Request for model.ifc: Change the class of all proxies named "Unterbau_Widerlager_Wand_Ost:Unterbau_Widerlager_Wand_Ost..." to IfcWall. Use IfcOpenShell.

First a look at what the model holds.

```python
import re

import ifcopenshell

model = ifcopenshell.open("model.ifc")
print(model.schema)
seen = {}
for e in model.by_type("IfcBuildingElementProxy"):
    name = re.sub(r":\d+(:\d+)?$", "", e.Name or "")  # drop the element id that some exporters append
    seen[name] = seen.get(name, 0) + 1
for name, count in sorted(seen.items()):
    print(count, "x", name)
```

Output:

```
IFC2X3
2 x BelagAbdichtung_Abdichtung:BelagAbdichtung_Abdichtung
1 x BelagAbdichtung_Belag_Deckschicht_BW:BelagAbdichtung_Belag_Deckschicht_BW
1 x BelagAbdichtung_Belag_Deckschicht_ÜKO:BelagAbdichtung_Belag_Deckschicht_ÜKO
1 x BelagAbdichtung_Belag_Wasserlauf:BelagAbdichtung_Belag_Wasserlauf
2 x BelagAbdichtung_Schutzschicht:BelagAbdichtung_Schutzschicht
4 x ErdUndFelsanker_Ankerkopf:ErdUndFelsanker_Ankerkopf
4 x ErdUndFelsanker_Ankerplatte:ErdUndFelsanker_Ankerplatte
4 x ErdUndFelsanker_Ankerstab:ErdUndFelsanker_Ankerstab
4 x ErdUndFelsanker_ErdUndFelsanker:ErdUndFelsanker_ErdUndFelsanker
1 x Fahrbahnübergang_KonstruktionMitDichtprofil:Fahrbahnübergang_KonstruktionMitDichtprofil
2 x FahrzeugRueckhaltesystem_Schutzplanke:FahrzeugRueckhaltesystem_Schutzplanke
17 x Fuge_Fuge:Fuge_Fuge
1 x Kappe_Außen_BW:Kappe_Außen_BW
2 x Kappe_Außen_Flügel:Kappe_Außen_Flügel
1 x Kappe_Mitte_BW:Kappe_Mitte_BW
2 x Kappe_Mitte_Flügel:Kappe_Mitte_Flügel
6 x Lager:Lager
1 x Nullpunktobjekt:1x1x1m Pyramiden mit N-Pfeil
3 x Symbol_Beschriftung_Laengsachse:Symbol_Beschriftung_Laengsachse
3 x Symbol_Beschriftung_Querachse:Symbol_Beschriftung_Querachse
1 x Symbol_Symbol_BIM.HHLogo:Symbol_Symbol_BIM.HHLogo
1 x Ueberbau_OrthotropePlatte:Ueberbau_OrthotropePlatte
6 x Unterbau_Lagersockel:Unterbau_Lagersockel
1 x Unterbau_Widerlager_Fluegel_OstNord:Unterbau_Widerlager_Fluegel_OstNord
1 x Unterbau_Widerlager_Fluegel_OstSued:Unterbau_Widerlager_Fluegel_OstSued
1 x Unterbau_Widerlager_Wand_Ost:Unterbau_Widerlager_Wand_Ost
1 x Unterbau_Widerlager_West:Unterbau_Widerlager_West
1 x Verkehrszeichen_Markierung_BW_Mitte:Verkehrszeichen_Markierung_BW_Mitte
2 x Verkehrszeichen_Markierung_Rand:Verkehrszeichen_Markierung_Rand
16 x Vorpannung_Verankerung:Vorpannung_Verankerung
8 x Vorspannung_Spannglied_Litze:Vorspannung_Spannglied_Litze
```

```python
import ifcopenshell
import ifcopenshell.api.root

model = ifcopenshell.open("model.ifc")

proxies = [e.id() for e in model.by_type("IfcBuildingElementProxy") if (e.Name or "").startswith("Unterbau_Widerlager_Wand_Ost:Unterbau_Widerlager_Wand_Ost")]
for step_id in proxies:
    proxy = model.by_id(step_id)
    # Reclassifying a typed element also reclassifies its type and the type's other occurrences.
    if proxy.is_a("IfcBuildingElementProxy"):
        ifcopenshell.api.root.reassign_class(model, product=proxy, ifc_class="IfcWall")

print(sum(model.by_id(i).is_a("IfcWall") for i in proxies), "reclassified")

model.write("model_edited.ifc")
```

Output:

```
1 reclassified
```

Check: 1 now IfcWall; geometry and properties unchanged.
